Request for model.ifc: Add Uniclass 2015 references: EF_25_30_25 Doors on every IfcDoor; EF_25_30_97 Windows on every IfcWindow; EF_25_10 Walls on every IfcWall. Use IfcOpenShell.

First a look at what the model holds.

```python
import ifcopenshell

model = ifcopenshell.open("model.ifc")
print(model.schema)
print("classifications:", [c.Name for c in model.by_type("IfcClassification")])
for ifc_class in ("IfcDoor", "IfcRoof", "IfcStair", "IfcWall", "IfcWindow"):
    print(ifc_class, len(model.by_type(ifc_class)))
```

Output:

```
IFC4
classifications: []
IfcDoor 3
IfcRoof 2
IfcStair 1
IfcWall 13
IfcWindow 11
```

```python
import ifcopenshell
import ifcopenshell.api.classification

model = ifcopenshell.open("model.ifc")

system = ifcopenshell.api.classification.add_classification(model, classification="Uniclass 2015")

codes = {
    "IfcDoor": ("EF_25_30_25", "Doors"),
    "IfcWindow": ("EF_25_30_97", "Windows"),
    "IfcWall": ("EF_25_10", "Walls"),
}
for ifc_class, (code, name) in codes.items():
    products = model.by_type(ifc_class)
    ifcopenshell.api.classification.add_reference(
        model, products=products, classification=system, identification=code, name=name
    )
    print(code, len(products))

model.write("model-out.ifc")
```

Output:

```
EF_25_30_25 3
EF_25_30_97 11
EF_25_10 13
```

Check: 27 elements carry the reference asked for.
